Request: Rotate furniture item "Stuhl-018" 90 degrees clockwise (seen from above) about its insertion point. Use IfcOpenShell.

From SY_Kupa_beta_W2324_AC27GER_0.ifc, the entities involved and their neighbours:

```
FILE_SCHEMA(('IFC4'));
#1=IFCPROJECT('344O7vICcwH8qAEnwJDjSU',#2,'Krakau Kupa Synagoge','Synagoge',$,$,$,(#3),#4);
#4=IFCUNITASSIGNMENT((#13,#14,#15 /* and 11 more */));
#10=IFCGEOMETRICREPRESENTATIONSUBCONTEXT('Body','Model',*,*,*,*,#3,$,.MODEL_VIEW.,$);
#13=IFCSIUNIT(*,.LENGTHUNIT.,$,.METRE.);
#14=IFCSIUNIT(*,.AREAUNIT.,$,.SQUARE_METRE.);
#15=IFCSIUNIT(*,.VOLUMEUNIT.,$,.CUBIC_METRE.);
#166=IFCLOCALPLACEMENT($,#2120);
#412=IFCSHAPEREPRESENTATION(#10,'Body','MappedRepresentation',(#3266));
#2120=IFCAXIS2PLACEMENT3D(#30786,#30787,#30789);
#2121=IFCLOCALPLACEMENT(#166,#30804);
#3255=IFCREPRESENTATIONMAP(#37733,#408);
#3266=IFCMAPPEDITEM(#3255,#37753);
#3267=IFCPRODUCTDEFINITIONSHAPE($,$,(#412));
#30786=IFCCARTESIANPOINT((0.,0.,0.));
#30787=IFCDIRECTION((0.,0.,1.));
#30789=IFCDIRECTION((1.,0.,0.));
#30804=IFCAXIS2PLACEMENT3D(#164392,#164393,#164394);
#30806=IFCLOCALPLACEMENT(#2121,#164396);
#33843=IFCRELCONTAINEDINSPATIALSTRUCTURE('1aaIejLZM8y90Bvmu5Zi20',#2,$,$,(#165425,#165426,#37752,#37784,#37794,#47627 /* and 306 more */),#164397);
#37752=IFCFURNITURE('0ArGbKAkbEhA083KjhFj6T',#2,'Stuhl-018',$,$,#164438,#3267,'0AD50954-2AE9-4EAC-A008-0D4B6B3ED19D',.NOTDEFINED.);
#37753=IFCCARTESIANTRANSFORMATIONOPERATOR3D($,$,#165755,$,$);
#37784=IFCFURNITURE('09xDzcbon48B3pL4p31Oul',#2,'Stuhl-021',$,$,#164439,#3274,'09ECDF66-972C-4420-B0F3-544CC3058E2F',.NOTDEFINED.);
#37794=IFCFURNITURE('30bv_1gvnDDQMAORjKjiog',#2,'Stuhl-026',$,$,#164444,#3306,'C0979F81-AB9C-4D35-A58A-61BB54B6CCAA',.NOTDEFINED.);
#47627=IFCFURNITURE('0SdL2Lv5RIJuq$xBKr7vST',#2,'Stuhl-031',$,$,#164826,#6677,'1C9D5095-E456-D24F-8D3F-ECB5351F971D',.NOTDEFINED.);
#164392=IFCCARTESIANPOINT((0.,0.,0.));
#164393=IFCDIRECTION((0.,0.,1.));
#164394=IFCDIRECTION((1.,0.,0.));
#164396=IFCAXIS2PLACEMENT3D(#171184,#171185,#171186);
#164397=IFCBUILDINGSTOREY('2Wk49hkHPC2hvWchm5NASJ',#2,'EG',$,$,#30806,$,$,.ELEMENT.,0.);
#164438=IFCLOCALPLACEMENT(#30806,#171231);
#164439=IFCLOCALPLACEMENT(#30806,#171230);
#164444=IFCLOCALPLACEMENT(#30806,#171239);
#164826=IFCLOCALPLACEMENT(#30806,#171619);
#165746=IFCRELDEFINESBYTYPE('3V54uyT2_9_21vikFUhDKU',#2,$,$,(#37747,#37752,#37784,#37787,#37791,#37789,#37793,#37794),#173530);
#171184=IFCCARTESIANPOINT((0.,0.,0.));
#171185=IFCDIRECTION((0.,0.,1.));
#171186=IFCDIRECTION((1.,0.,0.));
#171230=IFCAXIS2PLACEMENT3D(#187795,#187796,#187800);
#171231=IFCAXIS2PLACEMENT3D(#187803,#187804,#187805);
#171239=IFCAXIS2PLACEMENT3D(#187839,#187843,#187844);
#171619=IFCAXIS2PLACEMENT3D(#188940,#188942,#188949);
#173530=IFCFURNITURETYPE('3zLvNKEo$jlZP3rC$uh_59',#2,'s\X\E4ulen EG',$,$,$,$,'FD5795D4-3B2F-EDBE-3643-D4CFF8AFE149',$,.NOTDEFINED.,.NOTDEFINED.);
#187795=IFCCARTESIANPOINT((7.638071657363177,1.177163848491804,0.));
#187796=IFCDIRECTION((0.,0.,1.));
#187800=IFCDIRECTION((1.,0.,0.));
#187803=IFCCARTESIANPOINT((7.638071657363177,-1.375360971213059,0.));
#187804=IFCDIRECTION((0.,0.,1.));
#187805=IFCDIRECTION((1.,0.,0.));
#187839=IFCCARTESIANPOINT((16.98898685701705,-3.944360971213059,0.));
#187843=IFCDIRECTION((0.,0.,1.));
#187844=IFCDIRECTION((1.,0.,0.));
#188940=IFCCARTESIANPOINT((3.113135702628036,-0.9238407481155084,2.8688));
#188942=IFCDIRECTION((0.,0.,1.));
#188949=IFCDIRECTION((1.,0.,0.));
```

```python
import ifcopenshell
import ifcopenshell.api.geometry
import ifcopenshell.util.placement

model = ifcopenshell.open("SY_Kupa_beta_W2324_AC27GER_0.ifc")

item = model.by_guid("0ArGbKAkbEhA083KjhFj6T")
matrix = ifcopenshell.util.placement.get_local_placement(item.ObjectPlacement)
matrix = matrix @ ifcopenshell.util.placement.rotation(-90, "Z")
ifcopenshell.api.geometry.edit_object_placement(model, product=item, matrix=matrix, is_si=False)

print(ifcopenshell.util.placement.get_local_placement(item.ObjectPlacement).round(3) + 0.0)

model.write("SY_Kupa_beta_W2324_AC27GER_0_rev.ifc")
```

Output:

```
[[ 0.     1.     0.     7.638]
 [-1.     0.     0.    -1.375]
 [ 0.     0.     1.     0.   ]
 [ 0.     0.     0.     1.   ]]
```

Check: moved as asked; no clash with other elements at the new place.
